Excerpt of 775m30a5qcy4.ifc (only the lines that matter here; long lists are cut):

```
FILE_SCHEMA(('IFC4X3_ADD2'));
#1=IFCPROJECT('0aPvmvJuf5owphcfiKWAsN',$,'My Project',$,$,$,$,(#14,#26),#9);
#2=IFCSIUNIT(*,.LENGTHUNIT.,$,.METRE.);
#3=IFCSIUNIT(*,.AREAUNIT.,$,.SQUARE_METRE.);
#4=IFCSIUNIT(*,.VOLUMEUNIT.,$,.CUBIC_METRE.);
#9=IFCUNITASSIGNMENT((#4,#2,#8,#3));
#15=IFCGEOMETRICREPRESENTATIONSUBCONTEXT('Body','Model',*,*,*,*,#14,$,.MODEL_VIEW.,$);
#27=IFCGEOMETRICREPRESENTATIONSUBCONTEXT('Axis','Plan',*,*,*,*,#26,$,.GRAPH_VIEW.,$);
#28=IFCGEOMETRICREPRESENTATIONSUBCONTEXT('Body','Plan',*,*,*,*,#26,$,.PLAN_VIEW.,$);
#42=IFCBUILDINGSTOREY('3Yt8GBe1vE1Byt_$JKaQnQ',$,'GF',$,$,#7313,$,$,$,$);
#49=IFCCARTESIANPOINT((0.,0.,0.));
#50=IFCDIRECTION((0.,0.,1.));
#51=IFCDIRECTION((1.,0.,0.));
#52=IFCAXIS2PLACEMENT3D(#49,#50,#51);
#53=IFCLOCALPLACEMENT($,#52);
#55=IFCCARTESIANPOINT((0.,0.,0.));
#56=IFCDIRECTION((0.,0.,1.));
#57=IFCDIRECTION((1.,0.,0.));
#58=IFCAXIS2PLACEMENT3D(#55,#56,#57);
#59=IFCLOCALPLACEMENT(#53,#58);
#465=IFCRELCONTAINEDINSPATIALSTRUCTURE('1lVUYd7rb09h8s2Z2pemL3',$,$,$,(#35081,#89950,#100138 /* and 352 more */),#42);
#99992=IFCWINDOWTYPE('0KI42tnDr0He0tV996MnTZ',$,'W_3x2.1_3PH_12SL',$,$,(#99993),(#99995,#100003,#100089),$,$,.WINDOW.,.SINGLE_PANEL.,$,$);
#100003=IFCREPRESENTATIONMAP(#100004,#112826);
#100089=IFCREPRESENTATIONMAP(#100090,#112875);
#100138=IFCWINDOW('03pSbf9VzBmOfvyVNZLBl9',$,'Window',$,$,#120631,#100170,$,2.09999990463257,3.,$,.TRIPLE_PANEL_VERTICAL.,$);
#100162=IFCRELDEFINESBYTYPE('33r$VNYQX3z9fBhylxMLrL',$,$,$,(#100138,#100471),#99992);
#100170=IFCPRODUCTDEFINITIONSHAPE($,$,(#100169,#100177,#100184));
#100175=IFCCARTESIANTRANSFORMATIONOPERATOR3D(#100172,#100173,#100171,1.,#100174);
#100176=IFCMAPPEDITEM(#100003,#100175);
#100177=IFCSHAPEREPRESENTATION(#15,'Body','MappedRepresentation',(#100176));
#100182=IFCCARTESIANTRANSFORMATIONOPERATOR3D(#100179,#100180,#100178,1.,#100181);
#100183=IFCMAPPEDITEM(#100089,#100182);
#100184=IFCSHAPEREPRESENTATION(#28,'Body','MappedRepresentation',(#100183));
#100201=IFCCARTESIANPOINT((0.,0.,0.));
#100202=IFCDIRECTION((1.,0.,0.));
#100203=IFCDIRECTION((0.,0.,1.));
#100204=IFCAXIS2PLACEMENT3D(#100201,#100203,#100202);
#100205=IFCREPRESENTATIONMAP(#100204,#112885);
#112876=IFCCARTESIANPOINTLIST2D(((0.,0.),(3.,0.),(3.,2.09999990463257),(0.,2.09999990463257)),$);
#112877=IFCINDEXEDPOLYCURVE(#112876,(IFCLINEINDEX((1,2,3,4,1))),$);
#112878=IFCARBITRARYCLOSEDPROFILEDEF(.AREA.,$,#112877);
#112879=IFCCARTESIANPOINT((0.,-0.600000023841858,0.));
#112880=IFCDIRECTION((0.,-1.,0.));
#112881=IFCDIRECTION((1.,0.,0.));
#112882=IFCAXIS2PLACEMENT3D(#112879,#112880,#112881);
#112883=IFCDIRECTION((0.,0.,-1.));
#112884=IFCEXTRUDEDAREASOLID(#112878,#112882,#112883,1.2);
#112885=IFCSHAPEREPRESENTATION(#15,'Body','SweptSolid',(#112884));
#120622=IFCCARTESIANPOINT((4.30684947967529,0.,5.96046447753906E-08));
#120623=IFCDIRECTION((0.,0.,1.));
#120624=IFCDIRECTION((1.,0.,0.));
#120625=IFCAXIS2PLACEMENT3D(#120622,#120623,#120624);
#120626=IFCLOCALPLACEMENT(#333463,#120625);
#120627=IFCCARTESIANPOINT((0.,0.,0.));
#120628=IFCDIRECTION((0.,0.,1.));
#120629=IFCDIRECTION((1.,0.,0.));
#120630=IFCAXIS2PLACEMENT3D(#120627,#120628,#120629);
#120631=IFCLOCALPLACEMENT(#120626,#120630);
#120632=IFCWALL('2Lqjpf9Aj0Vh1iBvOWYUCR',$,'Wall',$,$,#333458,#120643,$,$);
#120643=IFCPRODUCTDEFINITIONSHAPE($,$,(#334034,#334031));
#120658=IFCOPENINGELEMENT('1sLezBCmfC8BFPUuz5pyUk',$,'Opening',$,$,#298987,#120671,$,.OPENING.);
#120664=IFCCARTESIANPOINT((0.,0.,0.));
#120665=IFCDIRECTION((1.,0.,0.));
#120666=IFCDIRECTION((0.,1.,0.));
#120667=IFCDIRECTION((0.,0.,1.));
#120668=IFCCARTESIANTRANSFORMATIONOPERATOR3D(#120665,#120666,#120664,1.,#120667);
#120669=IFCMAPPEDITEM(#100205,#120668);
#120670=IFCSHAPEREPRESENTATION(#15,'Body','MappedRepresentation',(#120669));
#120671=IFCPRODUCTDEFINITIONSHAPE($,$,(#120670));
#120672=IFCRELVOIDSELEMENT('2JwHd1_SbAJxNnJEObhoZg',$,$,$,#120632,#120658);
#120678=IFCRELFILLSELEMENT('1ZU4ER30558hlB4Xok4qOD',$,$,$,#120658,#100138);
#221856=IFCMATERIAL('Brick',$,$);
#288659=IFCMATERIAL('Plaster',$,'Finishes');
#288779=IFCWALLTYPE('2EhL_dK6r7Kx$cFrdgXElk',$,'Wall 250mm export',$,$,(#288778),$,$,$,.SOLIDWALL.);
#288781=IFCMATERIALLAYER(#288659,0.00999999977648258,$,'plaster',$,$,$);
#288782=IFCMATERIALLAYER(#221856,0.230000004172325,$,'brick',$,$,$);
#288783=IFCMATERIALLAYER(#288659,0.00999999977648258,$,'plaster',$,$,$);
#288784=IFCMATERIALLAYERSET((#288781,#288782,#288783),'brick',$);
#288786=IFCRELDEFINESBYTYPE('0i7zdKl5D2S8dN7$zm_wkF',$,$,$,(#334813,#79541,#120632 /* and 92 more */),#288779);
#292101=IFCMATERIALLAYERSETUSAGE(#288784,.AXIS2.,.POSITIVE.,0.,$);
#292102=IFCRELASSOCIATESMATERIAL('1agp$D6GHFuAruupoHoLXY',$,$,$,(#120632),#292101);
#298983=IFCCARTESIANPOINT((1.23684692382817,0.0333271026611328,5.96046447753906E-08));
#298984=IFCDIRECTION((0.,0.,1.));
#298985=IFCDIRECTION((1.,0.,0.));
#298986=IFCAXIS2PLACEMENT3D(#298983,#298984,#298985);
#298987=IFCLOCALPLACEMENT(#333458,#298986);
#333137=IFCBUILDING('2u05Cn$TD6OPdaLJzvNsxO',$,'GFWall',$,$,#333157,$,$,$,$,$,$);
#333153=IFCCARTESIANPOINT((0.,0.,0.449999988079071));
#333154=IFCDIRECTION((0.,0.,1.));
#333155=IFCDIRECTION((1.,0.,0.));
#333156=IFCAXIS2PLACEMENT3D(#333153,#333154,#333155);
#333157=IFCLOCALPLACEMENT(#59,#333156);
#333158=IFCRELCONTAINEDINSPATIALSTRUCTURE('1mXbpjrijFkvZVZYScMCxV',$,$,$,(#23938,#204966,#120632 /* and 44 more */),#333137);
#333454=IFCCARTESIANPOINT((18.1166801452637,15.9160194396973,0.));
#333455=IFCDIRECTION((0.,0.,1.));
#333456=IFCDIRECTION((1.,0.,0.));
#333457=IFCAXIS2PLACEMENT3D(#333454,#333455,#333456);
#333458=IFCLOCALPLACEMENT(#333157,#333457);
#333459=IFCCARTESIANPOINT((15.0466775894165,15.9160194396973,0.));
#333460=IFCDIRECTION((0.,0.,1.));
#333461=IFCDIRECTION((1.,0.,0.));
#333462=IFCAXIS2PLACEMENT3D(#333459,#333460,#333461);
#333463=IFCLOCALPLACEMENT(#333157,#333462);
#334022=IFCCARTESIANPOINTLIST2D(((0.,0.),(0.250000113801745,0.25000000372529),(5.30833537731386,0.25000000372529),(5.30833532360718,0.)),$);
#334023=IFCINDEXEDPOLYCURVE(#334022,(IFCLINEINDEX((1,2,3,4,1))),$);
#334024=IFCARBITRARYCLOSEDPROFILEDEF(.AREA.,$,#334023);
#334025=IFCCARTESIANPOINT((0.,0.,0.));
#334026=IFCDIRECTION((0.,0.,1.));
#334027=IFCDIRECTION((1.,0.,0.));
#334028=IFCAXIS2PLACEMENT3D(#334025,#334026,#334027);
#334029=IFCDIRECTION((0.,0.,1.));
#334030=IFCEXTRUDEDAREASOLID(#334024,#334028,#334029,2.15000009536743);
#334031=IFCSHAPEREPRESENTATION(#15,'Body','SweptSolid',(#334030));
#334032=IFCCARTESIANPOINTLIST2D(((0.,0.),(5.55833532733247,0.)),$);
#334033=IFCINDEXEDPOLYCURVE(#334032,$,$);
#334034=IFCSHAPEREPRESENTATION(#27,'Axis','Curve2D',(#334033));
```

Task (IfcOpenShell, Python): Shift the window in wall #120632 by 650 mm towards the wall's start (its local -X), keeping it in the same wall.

```python
import ifcopenshell
import ifcopenshell.api.geometry
import ifcopenshell.util.placement

model = ifcopenshell.open("775m30a5qcy4.ifc")

window = model.by_guid("03pSbf9VzBmOfvyVNZLBl9")
opening = window.FillsVoids[0].RelatingOpeningElement
wall = opening.VoidsElements[0].RelatingBuildingElement

wall_matrix = ifcopenshell.util.placement.get_local_placement(wall.ObjectPlacement)
shift = wall_matrix[:3, 0] * -0.65
before = ifcopenshell.util.placement.get_local_placement(window.ObjectPlacement)[:3, 3].copy()

# The window is not placed relative to its opening, so move both.
for product in (opening, window):
    matrix = ifcopenshell.util.placement.get_local_placement(product.ObjectPlacement)
    matrix[:3, 3] += shift
    ifcopenshell.api.geometry.edit_object_placement(model, product=product, matrix=matrix, is_si=False)

after = ifcopenshell.util.placement.get_local_placement(window.ObjectPlacement)[:3, 3]
print("window moved by", (after - before).round(3) + 0.0)

model.write("775m30a5qcy4_rev.ifc")
```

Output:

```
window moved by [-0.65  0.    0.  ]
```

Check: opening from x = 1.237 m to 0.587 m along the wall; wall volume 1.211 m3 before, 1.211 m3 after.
